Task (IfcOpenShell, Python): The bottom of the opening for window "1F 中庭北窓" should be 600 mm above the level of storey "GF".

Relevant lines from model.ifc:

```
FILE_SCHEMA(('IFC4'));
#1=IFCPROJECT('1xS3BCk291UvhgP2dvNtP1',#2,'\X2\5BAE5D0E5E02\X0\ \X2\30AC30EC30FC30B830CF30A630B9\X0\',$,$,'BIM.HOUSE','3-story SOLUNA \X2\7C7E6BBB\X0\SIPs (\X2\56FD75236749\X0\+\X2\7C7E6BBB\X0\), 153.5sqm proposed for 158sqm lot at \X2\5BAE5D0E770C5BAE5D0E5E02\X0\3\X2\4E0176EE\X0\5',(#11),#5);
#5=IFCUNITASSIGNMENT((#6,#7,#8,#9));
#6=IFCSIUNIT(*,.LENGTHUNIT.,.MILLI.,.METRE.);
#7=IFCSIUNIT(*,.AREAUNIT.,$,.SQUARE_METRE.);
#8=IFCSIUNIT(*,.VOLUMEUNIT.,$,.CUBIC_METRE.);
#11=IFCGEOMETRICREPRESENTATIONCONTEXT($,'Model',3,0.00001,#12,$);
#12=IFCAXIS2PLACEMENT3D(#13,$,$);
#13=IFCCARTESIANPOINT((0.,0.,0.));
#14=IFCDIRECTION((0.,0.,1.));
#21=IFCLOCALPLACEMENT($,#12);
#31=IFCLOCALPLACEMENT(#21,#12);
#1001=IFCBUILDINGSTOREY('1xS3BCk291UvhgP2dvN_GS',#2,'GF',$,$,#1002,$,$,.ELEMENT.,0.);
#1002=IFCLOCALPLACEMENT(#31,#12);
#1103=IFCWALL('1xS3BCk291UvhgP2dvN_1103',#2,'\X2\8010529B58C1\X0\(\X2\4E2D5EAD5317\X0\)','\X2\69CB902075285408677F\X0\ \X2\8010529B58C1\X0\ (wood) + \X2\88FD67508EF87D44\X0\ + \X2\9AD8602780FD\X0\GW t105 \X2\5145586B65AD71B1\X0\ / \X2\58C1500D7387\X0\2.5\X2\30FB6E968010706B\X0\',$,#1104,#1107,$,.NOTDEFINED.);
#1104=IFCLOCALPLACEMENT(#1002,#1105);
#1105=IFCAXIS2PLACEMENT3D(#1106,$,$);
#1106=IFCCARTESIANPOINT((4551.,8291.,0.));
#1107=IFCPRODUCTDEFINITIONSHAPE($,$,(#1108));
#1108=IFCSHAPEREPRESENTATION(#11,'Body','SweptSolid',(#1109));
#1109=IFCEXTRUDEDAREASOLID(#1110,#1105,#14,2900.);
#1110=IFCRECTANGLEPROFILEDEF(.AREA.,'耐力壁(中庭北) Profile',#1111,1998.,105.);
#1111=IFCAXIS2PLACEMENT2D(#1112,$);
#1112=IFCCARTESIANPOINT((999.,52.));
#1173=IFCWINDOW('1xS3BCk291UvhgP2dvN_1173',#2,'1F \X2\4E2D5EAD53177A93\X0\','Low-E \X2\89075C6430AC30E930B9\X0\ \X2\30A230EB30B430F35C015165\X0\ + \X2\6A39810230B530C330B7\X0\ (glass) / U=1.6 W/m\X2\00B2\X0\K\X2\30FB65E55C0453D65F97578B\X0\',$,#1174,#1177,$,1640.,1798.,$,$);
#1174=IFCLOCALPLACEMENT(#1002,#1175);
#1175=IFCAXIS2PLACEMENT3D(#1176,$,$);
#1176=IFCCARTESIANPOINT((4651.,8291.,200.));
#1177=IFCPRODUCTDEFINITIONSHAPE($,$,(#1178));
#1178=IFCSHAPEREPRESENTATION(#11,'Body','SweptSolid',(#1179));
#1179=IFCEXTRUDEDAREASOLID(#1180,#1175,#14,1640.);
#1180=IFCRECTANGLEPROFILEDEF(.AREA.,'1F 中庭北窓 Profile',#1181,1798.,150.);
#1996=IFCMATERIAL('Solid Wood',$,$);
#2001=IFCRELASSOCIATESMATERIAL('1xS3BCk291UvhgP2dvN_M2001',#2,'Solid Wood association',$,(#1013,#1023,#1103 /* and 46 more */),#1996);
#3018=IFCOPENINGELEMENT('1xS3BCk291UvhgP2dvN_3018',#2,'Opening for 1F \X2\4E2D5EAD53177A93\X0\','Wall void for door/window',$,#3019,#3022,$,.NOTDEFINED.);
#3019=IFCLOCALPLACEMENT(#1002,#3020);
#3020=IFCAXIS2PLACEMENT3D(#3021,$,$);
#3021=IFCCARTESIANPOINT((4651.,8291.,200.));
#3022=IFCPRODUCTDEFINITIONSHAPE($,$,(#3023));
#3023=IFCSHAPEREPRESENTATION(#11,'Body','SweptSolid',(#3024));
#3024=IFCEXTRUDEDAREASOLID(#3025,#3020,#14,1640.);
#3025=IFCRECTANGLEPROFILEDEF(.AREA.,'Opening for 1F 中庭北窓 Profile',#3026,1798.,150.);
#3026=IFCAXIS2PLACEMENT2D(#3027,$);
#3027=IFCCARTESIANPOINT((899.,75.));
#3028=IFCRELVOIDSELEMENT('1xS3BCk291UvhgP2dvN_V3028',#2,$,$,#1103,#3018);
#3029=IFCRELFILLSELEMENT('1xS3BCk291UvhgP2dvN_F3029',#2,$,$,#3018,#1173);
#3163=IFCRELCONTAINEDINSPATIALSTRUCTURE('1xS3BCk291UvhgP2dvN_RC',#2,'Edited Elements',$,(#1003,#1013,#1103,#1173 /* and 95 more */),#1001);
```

```python
import numpy as np
import ifcopenshell
import ifcopenshell.api.geometry
import ifcopenshell.geom
import ifcopenshell.util.element
import ifcopenshell.util.placement
import ifcopenshell.util.shape
import ifcopenshell.util.unit

model = ifcopenshell.open("model.ifc")
unit_scale = ifcopenshell.util.unit.calculate_unit_scale(model)

window = model.by_guid("1xS3BCk291UvhgP2dvN_1173")
opening = window.FillsVoids[0].RelatingOpeningElement
storey = ifcopenshell.util.element.get_container(window, ifc_class="IfcBuildingStorey")
level = ifcopenshell.util.placement.get_local_placement(storey.ObjectPlacement)[2, 3]

# The opening's origin need not be at the sill, so measure its lowest point.
shape = ifcopenshell.geom.create_shape(ifcopenshell.geom.settings(), opening)
bottom = ifcopenshell.util.shape.get_shape_bottom_elevation(shape, shape.geometry) / unit_scale
dz = level + 600.0 - bottom

shift = np.array([0.0, 0.0, dz])
# The window is not placed relative to its opening, so move both.
for product in (opening, window):
    matrix = ifcopenshell.util.placement.get_local_placement(product.ObjectPlacement)
    matrix[:3, 3] += shift
    ifcopenshell.api.geometry.edit_object_placement(model, product=product, matrix=matrix, is_si=False)

print(f"moved by {dz * unit_scale:+.3f} m")

model.write("model-out.ifc")
```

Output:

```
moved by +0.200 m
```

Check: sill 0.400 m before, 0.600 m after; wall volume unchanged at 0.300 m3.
